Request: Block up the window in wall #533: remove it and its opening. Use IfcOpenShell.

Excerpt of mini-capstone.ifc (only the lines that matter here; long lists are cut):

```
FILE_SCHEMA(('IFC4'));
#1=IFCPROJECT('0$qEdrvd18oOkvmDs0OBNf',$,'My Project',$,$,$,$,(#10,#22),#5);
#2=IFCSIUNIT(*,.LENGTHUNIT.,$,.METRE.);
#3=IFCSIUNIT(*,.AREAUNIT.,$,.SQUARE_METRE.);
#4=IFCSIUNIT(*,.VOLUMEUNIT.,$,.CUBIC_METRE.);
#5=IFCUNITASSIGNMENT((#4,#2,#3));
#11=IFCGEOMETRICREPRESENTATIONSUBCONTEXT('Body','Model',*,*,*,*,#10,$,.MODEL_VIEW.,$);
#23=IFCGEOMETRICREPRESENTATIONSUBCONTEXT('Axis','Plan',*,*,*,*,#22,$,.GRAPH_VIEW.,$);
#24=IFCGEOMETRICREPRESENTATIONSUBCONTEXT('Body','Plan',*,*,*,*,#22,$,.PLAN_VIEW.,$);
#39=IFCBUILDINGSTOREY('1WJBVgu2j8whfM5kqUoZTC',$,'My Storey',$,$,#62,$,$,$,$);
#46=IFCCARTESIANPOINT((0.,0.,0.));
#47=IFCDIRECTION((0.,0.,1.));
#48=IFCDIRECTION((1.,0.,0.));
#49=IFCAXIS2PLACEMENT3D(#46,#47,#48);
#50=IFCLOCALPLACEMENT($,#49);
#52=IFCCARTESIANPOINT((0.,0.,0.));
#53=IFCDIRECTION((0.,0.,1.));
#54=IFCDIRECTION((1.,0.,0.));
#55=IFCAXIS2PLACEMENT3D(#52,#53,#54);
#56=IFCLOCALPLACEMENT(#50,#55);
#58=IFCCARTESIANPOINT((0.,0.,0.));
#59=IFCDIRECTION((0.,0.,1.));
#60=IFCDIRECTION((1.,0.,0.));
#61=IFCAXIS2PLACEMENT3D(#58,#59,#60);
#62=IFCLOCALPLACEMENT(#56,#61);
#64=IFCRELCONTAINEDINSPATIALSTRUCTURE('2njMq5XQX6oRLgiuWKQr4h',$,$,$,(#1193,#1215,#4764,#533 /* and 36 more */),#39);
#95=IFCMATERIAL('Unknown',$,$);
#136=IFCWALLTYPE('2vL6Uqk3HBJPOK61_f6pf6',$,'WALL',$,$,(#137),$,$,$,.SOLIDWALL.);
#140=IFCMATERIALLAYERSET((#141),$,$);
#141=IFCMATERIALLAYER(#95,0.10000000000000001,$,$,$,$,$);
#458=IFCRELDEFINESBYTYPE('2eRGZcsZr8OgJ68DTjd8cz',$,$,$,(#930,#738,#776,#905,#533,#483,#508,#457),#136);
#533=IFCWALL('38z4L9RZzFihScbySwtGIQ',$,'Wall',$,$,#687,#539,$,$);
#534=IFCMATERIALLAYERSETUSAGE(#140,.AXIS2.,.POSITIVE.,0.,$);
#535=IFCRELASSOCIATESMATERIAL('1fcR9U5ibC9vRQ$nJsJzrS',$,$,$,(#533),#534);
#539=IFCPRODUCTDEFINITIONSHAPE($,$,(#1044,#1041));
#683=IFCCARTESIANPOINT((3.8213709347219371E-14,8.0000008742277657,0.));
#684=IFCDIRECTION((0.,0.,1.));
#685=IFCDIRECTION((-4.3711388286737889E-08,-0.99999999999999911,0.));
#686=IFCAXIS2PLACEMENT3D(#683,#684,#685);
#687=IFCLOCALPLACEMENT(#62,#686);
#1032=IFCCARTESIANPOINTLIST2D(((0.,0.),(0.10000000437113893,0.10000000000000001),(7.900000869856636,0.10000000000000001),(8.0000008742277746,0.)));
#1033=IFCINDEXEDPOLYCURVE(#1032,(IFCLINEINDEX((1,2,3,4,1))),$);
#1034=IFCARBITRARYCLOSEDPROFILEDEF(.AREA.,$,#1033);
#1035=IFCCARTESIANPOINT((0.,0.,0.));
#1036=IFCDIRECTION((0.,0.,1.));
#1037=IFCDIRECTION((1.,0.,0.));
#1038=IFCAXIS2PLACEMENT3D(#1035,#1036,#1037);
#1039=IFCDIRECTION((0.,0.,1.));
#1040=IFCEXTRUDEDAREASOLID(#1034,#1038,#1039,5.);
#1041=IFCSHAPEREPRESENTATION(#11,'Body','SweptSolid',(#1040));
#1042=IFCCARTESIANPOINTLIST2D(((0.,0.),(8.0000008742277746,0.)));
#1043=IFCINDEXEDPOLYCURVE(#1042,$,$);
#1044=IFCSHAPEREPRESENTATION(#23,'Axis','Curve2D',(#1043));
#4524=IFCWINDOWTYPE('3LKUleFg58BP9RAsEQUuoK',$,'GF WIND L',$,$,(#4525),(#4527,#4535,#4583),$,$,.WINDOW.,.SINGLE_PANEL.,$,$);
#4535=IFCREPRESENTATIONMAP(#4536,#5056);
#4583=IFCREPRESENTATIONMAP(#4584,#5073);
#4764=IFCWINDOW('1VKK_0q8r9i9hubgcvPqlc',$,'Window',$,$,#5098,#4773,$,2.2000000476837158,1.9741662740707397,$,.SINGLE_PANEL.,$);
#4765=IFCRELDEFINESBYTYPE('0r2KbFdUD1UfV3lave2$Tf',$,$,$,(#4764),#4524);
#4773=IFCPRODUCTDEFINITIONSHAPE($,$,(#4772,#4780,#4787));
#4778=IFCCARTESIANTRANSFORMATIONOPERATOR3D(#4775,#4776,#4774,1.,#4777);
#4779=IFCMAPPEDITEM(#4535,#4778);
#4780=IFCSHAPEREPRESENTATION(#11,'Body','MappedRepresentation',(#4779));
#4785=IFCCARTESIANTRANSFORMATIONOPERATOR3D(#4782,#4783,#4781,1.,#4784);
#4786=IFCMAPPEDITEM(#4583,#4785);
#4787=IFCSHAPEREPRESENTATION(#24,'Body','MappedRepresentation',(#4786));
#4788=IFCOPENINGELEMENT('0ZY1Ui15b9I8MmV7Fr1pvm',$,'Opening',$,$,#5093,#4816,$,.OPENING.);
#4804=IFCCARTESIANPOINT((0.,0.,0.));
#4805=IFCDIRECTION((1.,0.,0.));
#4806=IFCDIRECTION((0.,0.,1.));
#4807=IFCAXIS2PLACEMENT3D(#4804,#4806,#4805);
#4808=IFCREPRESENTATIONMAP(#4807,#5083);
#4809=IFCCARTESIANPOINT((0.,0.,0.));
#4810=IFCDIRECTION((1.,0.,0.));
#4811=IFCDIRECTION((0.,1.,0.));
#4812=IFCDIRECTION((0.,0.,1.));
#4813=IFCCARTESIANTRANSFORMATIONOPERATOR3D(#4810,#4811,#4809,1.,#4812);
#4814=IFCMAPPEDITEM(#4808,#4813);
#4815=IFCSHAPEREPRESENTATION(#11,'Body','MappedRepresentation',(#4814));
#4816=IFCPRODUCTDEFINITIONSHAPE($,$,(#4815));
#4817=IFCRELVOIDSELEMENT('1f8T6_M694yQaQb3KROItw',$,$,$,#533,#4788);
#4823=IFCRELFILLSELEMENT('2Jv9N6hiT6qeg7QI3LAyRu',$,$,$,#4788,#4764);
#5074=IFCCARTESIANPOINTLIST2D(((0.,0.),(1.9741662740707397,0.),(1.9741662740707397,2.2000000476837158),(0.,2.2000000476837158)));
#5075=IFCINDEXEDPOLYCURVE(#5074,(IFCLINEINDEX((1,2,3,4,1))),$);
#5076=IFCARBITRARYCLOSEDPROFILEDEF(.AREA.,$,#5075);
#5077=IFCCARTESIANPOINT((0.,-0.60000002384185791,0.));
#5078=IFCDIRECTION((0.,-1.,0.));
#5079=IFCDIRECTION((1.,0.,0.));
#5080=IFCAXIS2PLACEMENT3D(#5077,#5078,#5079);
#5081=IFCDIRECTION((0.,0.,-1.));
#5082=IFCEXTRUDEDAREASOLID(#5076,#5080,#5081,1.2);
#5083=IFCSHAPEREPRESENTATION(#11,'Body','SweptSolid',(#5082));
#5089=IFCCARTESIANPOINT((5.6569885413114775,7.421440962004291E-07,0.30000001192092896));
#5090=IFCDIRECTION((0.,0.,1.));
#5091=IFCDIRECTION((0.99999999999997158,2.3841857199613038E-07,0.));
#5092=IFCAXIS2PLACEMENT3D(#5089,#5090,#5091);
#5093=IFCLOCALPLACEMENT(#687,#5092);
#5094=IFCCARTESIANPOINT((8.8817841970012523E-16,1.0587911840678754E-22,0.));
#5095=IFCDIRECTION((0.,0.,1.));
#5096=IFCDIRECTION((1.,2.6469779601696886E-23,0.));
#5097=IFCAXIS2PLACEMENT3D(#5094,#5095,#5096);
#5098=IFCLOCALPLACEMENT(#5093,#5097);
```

```python
import ifcopenshell
import ifcopenshell.api.feature
import ifcopenshell.api.root
import ifcopenshell.geom
import ifcopenshell.util.shape

model = ifcopenshell.open("mini-capstone.ifc")
settings = ifcopenshell.geom.settings()


def volume(element):
    """Net volume in cubic metres, openings subtracted."""
    shape = ifcopenshell.geom.create_shape(settings, element)
    return ifcopenshell.util.shape.get_volume(shape.geometry)


window = model.by_guid("1VKK_0q8r9i9hubgcvPqlc")
opening = window.FillsVoids[0].RelatingOpeningElement
wall = opening.VoidsElements[0].RelatingBuildingElement
before = volume(wall)

ifcopenshell.api.root.remove_product(model, product=window)
ifcopenshell.api.feature.remove_feature(model, feature=opening)

after = volume(wall)

print(f"wall volume {before:.3f} -> {after:.3f} m3")

model.write("mini-capstone_edited.ifc")
```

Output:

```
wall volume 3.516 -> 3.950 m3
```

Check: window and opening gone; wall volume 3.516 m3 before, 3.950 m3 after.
